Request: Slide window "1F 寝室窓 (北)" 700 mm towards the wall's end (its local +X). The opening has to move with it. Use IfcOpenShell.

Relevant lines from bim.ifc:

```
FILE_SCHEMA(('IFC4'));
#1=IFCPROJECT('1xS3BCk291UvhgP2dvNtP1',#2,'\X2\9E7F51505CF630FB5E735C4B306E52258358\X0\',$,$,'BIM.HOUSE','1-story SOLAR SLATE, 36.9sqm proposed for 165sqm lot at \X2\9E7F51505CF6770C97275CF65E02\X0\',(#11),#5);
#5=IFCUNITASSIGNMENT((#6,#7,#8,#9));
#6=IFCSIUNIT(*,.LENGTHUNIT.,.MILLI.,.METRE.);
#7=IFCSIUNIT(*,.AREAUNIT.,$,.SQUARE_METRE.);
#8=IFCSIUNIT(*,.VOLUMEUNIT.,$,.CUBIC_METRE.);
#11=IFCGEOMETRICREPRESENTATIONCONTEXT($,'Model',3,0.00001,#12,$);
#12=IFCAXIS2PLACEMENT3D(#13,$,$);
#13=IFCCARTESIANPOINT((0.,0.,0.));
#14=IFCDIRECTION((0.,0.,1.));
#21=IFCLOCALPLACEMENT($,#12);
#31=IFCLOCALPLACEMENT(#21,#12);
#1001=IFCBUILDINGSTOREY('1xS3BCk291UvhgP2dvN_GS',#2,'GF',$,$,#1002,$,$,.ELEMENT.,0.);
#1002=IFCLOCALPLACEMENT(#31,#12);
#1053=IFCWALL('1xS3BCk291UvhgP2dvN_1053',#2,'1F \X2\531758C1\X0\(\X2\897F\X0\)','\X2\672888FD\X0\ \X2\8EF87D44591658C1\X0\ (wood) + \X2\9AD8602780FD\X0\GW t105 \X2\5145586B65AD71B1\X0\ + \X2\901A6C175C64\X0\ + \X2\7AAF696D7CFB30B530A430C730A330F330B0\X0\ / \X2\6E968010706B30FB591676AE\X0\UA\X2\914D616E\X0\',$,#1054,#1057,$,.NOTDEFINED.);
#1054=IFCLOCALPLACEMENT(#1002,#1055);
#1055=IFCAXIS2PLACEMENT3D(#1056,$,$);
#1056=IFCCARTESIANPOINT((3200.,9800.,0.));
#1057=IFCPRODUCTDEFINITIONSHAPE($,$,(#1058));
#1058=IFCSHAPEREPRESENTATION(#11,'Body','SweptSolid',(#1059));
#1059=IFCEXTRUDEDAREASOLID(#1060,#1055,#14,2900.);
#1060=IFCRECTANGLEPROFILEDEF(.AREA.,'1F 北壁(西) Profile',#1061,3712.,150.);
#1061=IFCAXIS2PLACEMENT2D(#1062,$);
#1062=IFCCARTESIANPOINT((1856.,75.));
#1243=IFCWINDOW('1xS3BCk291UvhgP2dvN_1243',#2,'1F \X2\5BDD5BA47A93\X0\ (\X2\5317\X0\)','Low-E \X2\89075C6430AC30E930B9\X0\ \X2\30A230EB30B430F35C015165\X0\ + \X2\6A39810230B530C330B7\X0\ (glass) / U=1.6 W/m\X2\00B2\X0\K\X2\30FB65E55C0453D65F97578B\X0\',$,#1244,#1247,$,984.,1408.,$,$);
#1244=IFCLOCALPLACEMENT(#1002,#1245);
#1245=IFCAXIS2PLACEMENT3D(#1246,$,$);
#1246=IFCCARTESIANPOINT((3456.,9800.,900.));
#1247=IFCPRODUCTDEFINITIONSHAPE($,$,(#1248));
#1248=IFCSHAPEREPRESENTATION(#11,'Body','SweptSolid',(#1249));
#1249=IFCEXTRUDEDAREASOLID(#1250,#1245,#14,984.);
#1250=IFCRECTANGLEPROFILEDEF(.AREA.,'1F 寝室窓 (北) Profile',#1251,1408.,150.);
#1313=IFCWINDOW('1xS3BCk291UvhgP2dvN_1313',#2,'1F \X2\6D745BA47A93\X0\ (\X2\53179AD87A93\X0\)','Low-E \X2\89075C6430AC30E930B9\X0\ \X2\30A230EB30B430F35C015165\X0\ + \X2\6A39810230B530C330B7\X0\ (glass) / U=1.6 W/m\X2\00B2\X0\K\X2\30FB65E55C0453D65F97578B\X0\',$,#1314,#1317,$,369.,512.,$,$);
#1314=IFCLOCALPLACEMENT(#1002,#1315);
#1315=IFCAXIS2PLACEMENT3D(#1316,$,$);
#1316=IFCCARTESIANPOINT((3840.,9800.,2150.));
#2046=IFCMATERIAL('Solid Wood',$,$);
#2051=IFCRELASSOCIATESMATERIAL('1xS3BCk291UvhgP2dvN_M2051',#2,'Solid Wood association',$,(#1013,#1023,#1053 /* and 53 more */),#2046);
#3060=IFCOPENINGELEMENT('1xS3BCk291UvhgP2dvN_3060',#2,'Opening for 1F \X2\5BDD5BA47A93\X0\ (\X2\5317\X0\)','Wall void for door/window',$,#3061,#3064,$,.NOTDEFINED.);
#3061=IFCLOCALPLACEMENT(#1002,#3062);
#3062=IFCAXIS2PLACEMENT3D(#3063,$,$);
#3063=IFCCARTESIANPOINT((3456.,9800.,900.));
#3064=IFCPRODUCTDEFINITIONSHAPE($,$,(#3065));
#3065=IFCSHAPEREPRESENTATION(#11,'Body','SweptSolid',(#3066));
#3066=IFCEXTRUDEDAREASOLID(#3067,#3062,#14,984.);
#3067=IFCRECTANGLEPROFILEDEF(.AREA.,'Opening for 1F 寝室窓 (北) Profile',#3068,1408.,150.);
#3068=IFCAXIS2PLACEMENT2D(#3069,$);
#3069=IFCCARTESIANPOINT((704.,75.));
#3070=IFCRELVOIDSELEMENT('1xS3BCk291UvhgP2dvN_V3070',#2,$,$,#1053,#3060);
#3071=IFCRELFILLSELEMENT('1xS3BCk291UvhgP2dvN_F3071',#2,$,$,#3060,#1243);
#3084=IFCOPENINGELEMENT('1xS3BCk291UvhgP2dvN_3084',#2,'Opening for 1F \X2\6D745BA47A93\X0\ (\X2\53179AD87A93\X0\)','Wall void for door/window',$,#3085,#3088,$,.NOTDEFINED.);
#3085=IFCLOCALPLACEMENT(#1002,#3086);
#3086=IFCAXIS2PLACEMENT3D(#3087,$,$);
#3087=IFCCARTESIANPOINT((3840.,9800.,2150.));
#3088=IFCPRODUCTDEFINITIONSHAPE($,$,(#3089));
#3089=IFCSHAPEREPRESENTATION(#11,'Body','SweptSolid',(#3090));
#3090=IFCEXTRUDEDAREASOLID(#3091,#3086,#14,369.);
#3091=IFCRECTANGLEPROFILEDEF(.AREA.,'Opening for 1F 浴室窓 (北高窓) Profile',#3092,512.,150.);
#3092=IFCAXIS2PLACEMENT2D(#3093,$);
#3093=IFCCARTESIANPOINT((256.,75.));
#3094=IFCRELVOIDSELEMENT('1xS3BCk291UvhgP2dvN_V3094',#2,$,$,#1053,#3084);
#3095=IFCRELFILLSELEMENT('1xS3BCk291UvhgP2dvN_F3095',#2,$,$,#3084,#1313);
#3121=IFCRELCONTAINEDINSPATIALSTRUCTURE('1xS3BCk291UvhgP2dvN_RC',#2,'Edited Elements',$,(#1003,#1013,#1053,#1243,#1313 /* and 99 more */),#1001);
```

```python
import ifcopenshell
import ifcopenshell.api.geometry
import ifcopenshell.util.placement

model = ifcopenshell.open("bim.ifc")

window = model.by_id(1243)
opening = window.FillsVoids[0].RelatingOpeningElement
wall = opening.VoidsElements[0].RelatingBuildingElement

wall_matrix = ifcopenshell.util.placement.get_local_placement(wall.ObjectPlacement)
shift = wall_matrix[:3, 0] * 700.0
before = ifcopenshell.util.placement.get_local_placement(window.ObjectPlacement)[:3, 3].copy()

# The window is not placed relative to its opening, so move both.
for product in (opening, window):
    matrix = ifcopenshell.util.placement.get_local_placement(product.ObjectPlacement)
    matrix[:3, 3] += shift
    ifcopenshell.api.geometry.edit_object_placement(model, product=product, matrix=matrix, is_si=False)

after = ifcopenshell.util.placement.get_local_placement(window.ObjectPlacement)[:3, 3]
print("window moved by", (after - before).round(3) + 0.0)

model.write("bim_rev.ifc")
```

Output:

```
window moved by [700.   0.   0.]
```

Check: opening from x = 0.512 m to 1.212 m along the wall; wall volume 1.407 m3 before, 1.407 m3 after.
